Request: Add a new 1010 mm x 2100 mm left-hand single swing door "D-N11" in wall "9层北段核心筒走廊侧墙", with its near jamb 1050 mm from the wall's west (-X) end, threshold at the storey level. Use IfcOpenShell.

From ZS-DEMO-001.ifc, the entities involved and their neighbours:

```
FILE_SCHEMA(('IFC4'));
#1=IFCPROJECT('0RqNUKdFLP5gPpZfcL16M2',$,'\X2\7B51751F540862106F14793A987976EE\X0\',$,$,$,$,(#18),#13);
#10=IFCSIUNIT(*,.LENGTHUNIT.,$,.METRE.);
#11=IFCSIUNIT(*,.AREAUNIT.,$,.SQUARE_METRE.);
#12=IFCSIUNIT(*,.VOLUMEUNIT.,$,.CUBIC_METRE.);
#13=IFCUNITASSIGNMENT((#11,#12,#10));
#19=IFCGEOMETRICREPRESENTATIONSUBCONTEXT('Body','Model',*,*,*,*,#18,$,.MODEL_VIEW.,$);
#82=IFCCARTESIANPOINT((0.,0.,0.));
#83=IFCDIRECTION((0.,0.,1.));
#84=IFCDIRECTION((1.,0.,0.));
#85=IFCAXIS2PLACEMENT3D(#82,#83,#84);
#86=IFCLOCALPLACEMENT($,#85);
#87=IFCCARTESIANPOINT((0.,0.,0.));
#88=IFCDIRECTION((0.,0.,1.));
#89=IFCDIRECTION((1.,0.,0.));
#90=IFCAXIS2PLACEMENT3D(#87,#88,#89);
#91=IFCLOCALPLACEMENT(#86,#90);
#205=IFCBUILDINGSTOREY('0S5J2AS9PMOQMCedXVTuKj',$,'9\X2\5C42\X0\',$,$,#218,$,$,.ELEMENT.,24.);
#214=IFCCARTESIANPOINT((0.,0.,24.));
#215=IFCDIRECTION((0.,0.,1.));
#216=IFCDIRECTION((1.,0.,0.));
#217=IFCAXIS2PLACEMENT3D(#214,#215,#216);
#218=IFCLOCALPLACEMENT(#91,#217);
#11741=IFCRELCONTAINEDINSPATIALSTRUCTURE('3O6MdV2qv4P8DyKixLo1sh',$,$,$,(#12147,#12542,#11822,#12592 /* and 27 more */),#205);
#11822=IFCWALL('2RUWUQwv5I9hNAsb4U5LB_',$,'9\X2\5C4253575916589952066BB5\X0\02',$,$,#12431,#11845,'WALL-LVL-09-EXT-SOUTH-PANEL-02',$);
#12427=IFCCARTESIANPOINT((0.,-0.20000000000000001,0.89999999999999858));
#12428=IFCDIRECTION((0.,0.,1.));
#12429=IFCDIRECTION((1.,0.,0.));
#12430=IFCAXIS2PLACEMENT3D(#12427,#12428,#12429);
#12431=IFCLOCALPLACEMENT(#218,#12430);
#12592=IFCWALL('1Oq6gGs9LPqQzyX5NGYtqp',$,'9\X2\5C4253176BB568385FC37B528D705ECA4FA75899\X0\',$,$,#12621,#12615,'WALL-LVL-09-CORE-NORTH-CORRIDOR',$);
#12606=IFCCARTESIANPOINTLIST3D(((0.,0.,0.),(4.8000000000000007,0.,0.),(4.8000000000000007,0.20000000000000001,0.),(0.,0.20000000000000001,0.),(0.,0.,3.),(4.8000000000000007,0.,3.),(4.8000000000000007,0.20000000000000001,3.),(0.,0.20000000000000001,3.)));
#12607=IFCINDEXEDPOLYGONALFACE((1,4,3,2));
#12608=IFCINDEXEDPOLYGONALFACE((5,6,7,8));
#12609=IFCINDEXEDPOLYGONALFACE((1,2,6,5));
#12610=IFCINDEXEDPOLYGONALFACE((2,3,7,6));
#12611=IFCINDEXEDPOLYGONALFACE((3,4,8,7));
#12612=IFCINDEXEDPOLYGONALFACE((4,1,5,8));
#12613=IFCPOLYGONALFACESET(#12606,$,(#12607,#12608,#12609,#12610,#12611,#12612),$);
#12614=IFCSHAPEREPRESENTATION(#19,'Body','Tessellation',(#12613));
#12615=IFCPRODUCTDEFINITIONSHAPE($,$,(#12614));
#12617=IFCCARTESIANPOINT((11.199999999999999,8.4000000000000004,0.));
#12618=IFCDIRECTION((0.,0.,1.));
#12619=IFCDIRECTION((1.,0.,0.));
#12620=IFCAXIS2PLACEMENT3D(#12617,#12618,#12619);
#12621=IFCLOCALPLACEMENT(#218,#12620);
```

```python
import numpy as np
import ifcopenshell
import ifcopenshell.api.feature
import ifcopenshell.api.geometry
import ifcopenshell.api.root
import ifcopenshell.api.spatial
import ifcopenshell.geom
import ifcopenshell.util.element
import ifcopenshell.util.placement
import ifcopenshell.util.representation
import ifcopenshell.util.shape
import ifcopenshell.util.unit

model = ifcopenshell.open("ZS-DEMO-001.ifc")
unit_scale = ifcopenshell.util.unit.calculate_unit_scale(model)
settings = ifcopenshell.geom.settings()


def volume(element):
    """Net volume in cubic metres, openings subtracted."""
    shape = ifcopenshell.geom.create_shape(settings, element)
    return ifcopenshell.util.shape.get_volume(shape.geometry)


wall = model.by_id(12592)
storey = ifcopenshell.util.element.get_container(wall, ifc_class="IfcBuildingStorey")
context = ifcopenshell.util.representation.get_context(model, "Model", "Body", "MODEL_VIEW")
before = volume(wall)

width, height, from_end, sill = 1.01, 2.1, 1.05, 0.0  # metres

# The wall runs along its own X axis, and the end named is its -X end.
wall_shape = ifcopenshell.geom.create_shape(settings, wall)
x, y, z = ifcopenshell.util.shape.get_vertices(wall_shape.geometry).T
start = x.min() + from_end
face, thickness = float(y.min()), float(y.max() - y.min())
wall_matrix = ifcopenshell.util.placement.get_local_placement(wall.ObjectPlacement)
level = ifcopenshell.util.placement.get_local_placement(storey.ObjectPlacement)[2, 3]


def in_wall(x, y):
    """Placement at x, y metres in the wall's axes, at sill height."""
    matrix = wall_matrix.copy()
    matrix[:, 3] = wall_matrix @ np.array([x / unit_scale, y / unit_scale, 0.0, 1.0])
    matrix[2, 3] = level + sill / unit_scale
    return matrix


# Opening: a box that overshoots both wall faces by 50 mm.
opening = ifcopenshell.api.root.create_entity(model, ifc_class="IfcOpeningElement", predefined_type="OPENING")
box = ifcopenshell.api.geometry.add_wall_representation(
    model, context=context, length=width, height=height, thickness=thickness + 0.1
)
ifcopenshell.api.geometry.assign_representation(model, product=opening, representation=box)
ifcopenshell.api.geometry.edit_object_placement(model, product=opening, matrix=in_wall(start, face - 0.05), is_si=False)
ifcopenshell.api.feature.add_feature(model, feature=opening, element=wall)

door = ifcopenshell.api.root.create_entity(model, ifc_class="IfcDoor", name="D-N11", predefined_type="DOOR")
door.OverallWidth, door.OverallHeight = width / unit_scale, height / unit_scale
door.OperationType = "SINGLE_SWING_LEFT"
body = ifcopenshell.api.geometry.add_door_representation(
    model,
    context=context,
    overall_width=door.OverallWidth,
    overall_height=door.OverallHeight,
    operation_type="SINGLE_SWING_LEFT",
    lining_properties={"LiningDepth": thickness / unit_scale, "ThresholdDepth": thickness / unit_scale},
)
ifcopenshell.api.geometry.assign_representation(model, product=door, representation=body)
ifcopenshell.api.spatial.assign_container(model, products=[door], relating_structure=storey)
ifcopenshell.api.feature.add_filling(model, opening=opening, element=door)

# The lining spans the wall, so the door starts at the wall face.
ifcopenshell.api.geometry.edit_object_placement(model, product=door, matrix=in_wall(start, face), is_si=False)

after = volume(wall)

print(f"wall volume {before:.3f} -> {after:.3f} m3")

model.write("ZS-DEMO-001-out.ifc")
```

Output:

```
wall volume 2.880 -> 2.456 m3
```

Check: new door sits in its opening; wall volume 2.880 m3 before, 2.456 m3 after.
